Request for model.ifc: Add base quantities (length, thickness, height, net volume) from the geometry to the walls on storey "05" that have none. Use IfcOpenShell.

First a look at what the model holds.

```python
import ifcopenshell
import ifcopenshell.util.element
import ifcopenshell.util.unit

model = ifcopenshell.open("model.ifc")
print(model.schema)
for unit_type in ("LENGTHUNIT", "AREAUNIT", "VOLUMEUNIT"):
    print(unit_type, ifcopenshell.util.unit.calculate_unit_scale(model, unit_type))
storey = next(s for s in model.by_type("IfcBuildingStorey") if s.Name == "05")
walls = [e for e in ifcopenshell.util.element.get_decomposition(storey) if e.is_a("IfcWall")]
for e in sorted(walls, key=lambda e: e.id()):
    print(e.id(), e.is_a(), e.Name, list(ifcopenshell.util.element.get_psets(e, qtos_only=True)), sep=" | ")
```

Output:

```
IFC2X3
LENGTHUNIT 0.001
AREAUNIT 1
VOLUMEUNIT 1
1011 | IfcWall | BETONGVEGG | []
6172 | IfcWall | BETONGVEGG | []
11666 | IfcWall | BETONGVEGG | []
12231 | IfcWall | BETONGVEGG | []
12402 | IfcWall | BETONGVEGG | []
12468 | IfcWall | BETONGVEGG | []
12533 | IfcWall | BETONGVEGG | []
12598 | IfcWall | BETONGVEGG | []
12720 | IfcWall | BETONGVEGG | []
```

```python
import ifcopenshell
import ifcopenshell.api.pset
import ifcopenshell.geom
import ifcopenshell.util.element
import ifcopenshell.util.shape
import ifcopenshell.util.unit

model = ifcopenshell.open("model.ifc")
unit_scale = ifcopenshell.util.unit.calculate_unit_scale(model)
volume_scale = ifcopenshell.util.unit.calculate_unit_scale(model, "VOLUMEUNIT")
settings = ifcopenshell.geom.settings()

storey = next(s for s in model.by_type("IfcBuildingStorey") if s.Name == "05")
walls = [e for e in ifcopenshell.util.element.get_decomposition(storey) if e.is_a("IfcWall")]

for e in sorted(walls, key=lambda e: e.id()):
    if ifcopenshell.util.element.get_psets(e, qtos_only=True, should_inherit=False):
        continue
    # Geometry comes back in metres, in the element's own axes.
    shape = ifcopenshell.geom.create_shape(settings, e)
    values = {
        "Length": ifcopenshell.util.shape.get_x(shape.geometry) / unit_scale,
        "Width": ifcopenshell.util.shape.get_y(shape.geometry) / unit_scale,
        "Height": ifcopenshell.util.shape.get_z(shape.geometry) / unit_scale,
        "NetVolume": ifcopenshell.util.shape.get_volume(shape.geometry) / volume_scale,
    }
    qto = ifcopenshell.api.pset.add_qto(model, product=e, name="BaseQuantities")
    ifcopenshell.api.pset.edit_qto(model, qto=qto, properties=values)
    print(e.id(), {k: round(v, 3) for k, v in values.items()})

model.write("model_edited.ifc")
```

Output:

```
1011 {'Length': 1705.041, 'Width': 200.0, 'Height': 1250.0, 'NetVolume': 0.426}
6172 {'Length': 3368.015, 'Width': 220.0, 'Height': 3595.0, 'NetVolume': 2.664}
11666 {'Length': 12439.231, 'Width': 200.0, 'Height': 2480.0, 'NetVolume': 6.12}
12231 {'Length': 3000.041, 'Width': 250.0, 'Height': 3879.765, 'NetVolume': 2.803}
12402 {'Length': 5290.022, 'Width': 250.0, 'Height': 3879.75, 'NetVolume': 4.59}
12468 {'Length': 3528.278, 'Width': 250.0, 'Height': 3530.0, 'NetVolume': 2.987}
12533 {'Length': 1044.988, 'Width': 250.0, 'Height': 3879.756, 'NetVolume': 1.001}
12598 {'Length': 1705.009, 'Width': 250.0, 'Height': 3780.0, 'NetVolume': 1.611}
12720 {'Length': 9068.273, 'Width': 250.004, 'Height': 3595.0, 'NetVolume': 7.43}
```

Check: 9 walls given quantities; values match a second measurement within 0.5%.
